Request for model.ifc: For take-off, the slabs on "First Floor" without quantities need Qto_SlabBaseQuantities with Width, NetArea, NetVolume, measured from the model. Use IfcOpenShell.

First a look at what the model holds.

```python
import ifcopenshell
import ifcopenshell.util.element
import ifcopenshell.util.unit

model = ifcopenshell.open("model.ifc")
print(model.schema)
for unit_type in ("LENGTHUNIT", "AREAUNIT", "VOLUMEUNIT"):
    print(unit_type, ifcopenshell.util.unit.calculate_unit_scale(model, unit_type))
storey = next(s for s in model.by_type("IfcBuildingStorey") if s.Name == "First Floor")
slabs = [e for e in ifcopenshell.util.element.get_decomposition(storey) if e.is_a("IfcSlab")]
for e in sorted(slabs, key=lambda e: e.id()):
    print(e.id(), e.is_a(), e.Name, list(ifcopenshell.util.element.get_psets(e, qtos_only=True)), sep=" | ")
```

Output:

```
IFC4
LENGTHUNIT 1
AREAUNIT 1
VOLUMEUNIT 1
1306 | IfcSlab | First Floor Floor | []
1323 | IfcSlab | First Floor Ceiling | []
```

```python
import ifcopenshell
import ifcopenshell.api.pset
import ifcopenshell.geom
import ifcopenshell.util.element
import ifcopenshell.util.shape
import ifcopenshell.util.unit

model = ifcopenshell.open("model.ifc")
unit_scale = ifcopenshell.util.unit.calculate_unit_scale(model)
area_scale = ifcopenshell.util.unit.calculate_unit_scale(model, "AREAUNIT")
volume_scale = ifcopenshell.util.unit.calculate_unit_scale(model, "VOLUMEUNIT")
settings = ifcopenshell.geom.settings()

storey = next(s for s in model.by_type("IfcBuildingStorey") if s.Name == "First Floor")
slabs = [e for e in ifcopenshell.util.element.get_decomposition(storey) if e.is_a("IfcSlab")]

for e in sorted(slabs, key=lambda e: e.id()):
    if ifcopenshell.util.element.get_psets(e, qtos_only=True, should_inherit=False):
        continue
    # Geometry comes back in metres, in the element's own axes.
    shape = ifcopenshell.geom.create_shape(settings, e)
    values = {
        "Width": ifcopenshell.util.shape.get_z(shape.geometry) / unit_scale,
        "NetArea": ifcopenshell.util.shape.get_footprint_area(shape.geometry) / area_scale,
        "NetVolume": ifcopenshell.util.shape.get_volume(shape.geometry) / volume_scale,
    }
    qto = ifcopenshell.api.pset.add_qto(model, product=e, name="Qto_SlabBaseQuantities")
    ifcopenshell.api.pset.edit_qto(model, qto=qto, properties=values)
    print(e.id(), {k: round(v, 3) for k, v in values.items()})

model.write("model_v2.ifc")
```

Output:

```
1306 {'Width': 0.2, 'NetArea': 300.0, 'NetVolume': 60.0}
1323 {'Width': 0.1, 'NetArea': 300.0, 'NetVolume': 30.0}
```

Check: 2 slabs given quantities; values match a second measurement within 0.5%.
